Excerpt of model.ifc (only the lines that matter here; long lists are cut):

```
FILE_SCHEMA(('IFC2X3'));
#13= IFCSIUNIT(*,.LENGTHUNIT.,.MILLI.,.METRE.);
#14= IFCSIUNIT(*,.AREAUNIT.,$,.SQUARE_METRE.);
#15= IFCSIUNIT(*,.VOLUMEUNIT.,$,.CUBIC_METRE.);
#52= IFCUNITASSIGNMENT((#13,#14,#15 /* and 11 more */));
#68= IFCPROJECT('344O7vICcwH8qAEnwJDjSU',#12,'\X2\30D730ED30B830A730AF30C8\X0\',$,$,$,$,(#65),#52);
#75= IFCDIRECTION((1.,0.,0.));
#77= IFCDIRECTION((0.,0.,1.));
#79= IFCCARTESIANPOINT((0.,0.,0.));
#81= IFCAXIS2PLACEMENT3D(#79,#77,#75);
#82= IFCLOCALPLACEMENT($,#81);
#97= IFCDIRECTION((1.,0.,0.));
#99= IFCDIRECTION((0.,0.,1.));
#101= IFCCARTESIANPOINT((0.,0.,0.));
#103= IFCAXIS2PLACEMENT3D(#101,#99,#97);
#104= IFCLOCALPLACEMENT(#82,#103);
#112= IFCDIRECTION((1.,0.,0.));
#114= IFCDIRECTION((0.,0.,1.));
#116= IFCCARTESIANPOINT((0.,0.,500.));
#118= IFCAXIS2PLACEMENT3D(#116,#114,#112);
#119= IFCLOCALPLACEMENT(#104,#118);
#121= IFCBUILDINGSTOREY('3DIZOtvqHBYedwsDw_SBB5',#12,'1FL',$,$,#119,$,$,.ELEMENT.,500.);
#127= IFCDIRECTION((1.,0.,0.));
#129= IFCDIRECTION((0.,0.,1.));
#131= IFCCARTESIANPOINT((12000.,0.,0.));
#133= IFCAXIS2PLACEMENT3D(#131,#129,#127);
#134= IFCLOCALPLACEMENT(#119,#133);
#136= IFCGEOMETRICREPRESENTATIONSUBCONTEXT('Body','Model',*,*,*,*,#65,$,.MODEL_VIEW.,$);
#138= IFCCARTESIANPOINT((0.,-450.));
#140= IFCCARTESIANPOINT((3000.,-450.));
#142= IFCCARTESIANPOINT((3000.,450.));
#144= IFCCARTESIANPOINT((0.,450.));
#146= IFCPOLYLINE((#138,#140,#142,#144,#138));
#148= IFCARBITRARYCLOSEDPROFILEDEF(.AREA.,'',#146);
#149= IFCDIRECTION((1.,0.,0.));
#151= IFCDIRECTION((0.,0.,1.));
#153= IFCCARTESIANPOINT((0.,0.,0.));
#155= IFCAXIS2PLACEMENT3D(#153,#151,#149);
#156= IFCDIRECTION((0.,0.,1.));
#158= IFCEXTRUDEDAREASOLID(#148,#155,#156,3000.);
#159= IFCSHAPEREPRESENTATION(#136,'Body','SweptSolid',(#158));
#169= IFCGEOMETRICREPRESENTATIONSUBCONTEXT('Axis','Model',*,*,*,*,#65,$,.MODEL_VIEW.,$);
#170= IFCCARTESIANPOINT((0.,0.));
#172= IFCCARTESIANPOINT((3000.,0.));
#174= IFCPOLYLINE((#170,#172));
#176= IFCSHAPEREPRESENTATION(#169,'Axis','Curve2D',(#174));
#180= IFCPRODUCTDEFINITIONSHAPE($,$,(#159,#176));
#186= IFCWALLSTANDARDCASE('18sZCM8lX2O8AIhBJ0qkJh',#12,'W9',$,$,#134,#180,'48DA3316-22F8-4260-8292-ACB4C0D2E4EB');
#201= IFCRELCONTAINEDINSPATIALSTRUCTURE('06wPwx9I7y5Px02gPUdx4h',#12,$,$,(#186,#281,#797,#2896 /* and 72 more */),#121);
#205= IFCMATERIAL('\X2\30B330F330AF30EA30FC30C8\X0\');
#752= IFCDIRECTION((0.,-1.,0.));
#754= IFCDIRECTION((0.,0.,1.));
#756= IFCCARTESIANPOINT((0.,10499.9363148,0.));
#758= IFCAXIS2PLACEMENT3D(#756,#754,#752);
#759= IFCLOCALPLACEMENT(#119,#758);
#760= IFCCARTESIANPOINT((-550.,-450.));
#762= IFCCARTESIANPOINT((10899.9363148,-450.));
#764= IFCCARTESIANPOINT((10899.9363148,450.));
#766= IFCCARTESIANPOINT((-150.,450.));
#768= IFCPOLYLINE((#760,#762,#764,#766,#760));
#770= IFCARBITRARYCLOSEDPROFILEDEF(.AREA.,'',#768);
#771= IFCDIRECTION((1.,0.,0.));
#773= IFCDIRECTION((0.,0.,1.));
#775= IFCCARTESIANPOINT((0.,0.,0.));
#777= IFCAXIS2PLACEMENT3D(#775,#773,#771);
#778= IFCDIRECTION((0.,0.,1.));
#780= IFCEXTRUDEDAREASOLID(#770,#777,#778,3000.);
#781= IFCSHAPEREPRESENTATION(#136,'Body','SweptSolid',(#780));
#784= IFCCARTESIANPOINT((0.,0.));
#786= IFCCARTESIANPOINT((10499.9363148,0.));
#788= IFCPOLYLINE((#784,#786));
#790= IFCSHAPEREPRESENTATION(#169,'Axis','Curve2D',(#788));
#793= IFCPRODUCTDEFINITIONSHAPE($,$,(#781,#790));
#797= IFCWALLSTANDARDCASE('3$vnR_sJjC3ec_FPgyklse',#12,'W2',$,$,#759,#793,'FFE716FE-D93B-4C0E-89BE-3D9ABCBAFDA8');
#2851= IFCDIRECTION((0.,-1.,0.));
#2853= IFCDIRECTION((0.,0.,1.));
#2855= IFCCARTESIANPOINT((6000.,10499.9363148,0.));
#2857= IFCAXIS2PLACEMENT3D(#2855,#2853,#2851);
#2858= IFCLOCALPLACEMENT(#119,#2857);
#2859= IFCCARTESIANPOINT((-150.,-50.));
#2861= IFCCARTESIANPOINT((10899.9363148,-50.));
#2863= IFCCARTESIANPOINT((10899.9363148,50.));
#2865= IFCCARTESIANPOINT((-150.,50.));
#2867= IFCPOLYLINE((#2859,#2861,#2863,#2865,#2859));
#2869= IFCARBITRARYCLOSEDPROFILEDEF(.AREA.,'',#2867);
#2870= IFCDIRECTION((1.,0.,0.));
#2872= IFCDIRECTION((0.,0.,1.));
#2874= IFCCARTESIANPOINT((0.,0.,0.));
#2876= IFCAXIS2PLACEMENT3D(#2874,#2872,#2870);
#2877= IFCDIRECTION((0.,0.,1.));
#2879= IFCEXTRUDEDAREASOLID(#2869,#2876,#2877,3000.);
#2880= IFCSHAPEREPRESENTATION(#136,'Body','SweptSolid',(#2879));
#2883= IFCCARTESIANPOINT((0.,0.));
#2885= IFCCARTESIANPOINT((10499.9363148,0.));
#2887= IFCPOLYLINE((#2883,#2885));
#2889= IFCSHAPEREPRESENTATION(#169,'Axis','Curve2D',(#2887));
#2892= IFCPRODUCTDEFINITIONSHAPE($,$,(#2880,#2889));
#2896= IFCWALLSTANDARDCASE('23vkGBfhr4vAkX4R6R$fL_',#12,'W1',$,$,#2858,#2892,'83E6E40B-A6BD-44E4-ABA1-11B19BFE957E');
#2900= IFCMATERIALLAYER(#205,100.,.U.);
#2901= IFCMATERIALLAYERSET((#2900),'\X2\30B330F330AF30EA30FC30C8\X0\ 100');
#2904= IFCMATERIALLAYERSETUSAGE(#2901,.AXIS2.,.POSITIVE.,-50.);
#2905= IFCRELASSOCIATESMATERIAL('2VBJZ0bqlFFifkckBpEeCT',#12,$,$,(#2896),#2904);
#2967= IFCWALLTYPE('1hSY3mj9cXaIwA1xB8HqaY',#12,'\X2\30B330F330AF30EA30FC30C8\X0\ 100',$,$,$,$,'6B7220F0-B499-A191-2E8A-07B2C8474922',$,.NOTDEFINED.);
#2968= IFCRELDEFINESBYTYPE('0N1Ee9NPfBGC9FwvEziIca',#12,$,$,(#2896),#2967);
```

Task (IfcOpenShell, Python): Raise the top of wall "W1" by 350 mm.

```python
import ifcopenshell
import ifcopenshell.geom
import ifcopenshell.util.representation
import ifcopenshell.util.shape

model = ifcopenshell.open("model.ifc")
settings = ifcopenshell.geom.settings()


def volume(element):
    """Net volume in cubic metres, openings subtracted."""
    shape = ifcopenshell.geom.create_shape(settings, element)
    return ifcopenshell.util.shape.get_volume(shape.geometry)


wall = model.by_guid("23vkGBfhr4vAkX4R6R$fL_")
before = volume(wall)

body = ifcopenshell.util.representation.get_representation(wall, "Model", "Body")
solid = body.Items[0]
old_height = solid.Depth
solid.Depth += 350.0
after = volume(wall)

print(f"height {old_height:g} -> {solid.Depth:g}, volume {before:.3f} -> {after:.3f} m3")

model.write("model-out.ifc")
```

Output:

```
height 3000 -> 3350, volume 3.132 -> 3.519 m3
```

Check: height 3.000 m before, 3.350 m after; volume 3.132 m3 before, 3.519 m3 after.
